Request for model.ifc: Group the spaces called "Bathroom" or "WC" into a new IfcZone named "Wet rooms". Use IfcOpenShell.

First a look at what the model holds.

```python
import ifcopenshell

model = ifcopenshell.open("model.ifc")
print(model.schema)
seen = {}
for space in model.by_type("IfcSpace"):
    seen[space.LongName] = seen.get(space.LongName, 0) + 1
for name, count in sorted(seen.items(), key=str):
    print(count, "x", name)
print("zones:", [z.Name for z in model.by_type("IfcZone")][:20])
```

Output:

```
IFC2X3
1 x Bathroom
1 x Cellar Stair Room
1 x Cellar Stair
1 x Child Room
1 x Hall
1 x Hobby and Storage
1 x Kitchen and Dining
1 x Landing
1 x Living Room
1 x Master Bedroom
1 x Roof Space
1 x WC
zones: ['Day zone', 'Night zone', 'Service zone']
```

```python
import ifcopenshell
import ifcopenshell.api.group
import ifcopenshell.api.root

model = ifcopenshell.open("model.ifc")

names = {"Bathroom", "WC"}
spaces = [s for s in model.by_type("IfcSpace") if s.LongName in names]

zone = ifcopenshell.api.root.create_entity(model, ifc_class="IfcZone", name="Wet rooms")
ifcopenshell.api.group.assign_group(model, products=spaces, group=zone)
print(len(spaces), "spaces in", zone.Name)

model.write("model-out.ifc")
```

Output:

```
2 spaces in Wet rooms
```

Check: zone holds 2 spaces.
